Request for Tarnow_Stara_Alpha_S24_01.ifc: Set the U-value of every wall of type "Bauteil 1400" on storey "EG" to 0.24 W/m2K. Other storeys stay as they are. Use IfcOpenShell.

First a look at what the model holds.

```python
import ifcopenshell
import ifcopenshell.util.element

model = ifcopenshell.open("Tarnow_Stara_Alpha_S24_01.ifc")
print(model.schema)
storey = next(s for s in model.by_type("IfcBuildingStorey") if s.Name == "EG")
walls = [e for e in ifcopenshell.util.element.get_decomposition(storey) if e.is_a("IfcWall")]
seen = {}
for e in walls:
    element_type = ifcopenshell.util.element.get_type(e)
    key = (element_type.Name if element_type != e and element_type else None, ifcopenshell.util.element.get_pset(e, "Pset_WallCommon", "ThermalTransmittance"))
    seen[key] = seen.get(key, 0) + 1
for (name, value), count in sorted(seen.items(), key=str):
    print(count, "x", name, "|", value)
```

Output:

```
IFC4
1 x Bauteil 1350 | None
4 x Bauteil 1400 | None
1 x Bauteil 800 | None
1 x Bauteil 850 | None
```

```python
import ifcopenshell
import ifcopenshell.api.pset
import ifcopenshell.util.element

model = ifcopenshell.open("Tarnow_Stara_Alpha_S24_01.ifc")

storey = next(s for s in model.by_type("IfcBuildingStorey") if s.Name == "EG")
walls = [e for e in ifcopenshell.util.element.get_decomposition(storey) if e.is_a("IfcWall")]

count = 0
for e in walls:
    element_type = ifcopenshell.util.element.get_type(e)
    if element_type in (None, e) or element_type.Name != "Bauteil 1400":
        continue
    # add_pset returns the element's existing set when there is one.
    pset = ifcopenshell.api.pset.add_pset(model, product=e, name="Pset_WallCommon")
    ifcopenshell.api.pset.edit_pset(model, pset=pset, properties={"ThermalTransmittance": 0.24})
    count += 1

print(count, "walls updated")

model.write("Tarnow_Stara_Alpha_S24_01_edited.ifc")
```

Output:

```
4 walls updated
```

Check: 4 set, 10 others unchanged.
